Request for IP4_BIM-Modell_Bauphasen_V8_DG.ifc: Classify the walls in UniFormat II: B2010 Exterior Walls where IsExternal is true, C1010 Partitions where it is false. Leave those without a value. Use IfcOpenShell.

First a look at what the model holds.

```python
import ifcopenshell
import ifcopenshell.util.element

model = ifcopenshell.open("IP4_BIM-Modell_Bauphasen_V8_DG.ifc")
print(model.schema)
print("classifications:", [c.Name for c in model.by_type("IfcClassification")])
values = [ifcopenshell.util.element.get_pset(e, "Pset_WallCommon", "IsExternal") for e in model.by_type("IfcWall")]
for value in (True, False, None):
    print("IsExternal", value, values.count(value))
```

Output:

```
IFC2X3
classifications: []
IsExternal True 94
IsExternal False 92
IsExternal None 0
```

```python
import ifcopenshell
import ifcopenshell.api.classification
import ifcopenshell.util.element

model = ifcopenshell.open("IP4_BIM-Modell_Bauphasen_V8_DG.ifc")

# IFC2X3 requires Source and Edition and has no link from the project to the system.
system = model.create_entity("IfcClassification", Source="ASTM", Edition="E1557", Name="UniFormat II")

walls = model.by_type("IfcWall")
external = {e: ifcopenshell.util.element.get_pset(e, "Pset_WallCommon", "IsExternal") for e in walls}
for flag, code, name in ((True, "B2010", "Exterior Walls"), (False, "C1010", "Partitions")):
    products = [e for e in walls if external[e] is flag]
    ifcopenshell.api.classification.add_reference(
        model, products=products, classification=system, identification=code, name=name
    )
    print(code, len(products))

model.write("IP4_BIM-Modell_Bauphasen_V8_DG_updated.ifc")
```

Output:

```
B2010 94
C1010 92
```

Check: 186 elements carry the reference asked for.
